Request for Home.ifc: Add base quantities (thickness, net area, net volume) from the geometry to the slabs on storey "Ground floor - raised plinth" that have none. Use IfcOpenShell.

First a look at what the model holds.

```python
import ifcopenshell
import ifcopenshell.util.element
import ifcopenshell.util.unit

model = ifcopenshell.open("Home.ifc")
print(model.schema)
for unit_type in ("LENGTHUNIT", "AREAUNIT", "VOLUMEUNIT"):
    print(unit_type, ifcopenshell.util.unit.calculate_unit_scale(model, unit_type))
storey = next(s for s in model.by_type("IfcBuildingStorey") if s.Name == "Ground floor - raised plinth")
slabs = [e for e in ifcopenshell.util.element.get_decomposition(storey) if e.is_a("IfcSlab")]
for e in sorted(slabs, key=lambda e: e.id()):
    print(e.id(), e.is_a(), e.Name, list(ifcopenshell.util.element.get_psets(e, qtos_only=True)), sep=" | ")
```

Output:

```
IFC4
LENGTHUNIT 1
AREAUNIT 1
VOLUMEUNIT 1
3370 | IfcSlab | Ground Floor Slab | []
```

```python
import ifcopenshell
import ifcopenshell.api.pset
import ifcopenshell.geom
import ifcopenshell.util.element
import ifcopenshell.util.shape
import ifcopenshell.util.unit

model = ifcopenshell.open("Home.ifc")
unit_scale = ifcopenshell.util.unit.calculate_unit_scale(model)
area_scale = ifcopenshell.util.unit.calculate_unit_scale(model, "AREAUNIT")
volume_scale = ifcopenshell.util.unit.calculate_unit_scale(model, "VOLUMEUNIT")
settings = ifcopenshell.geom.settings()

storey = next(s for s in model.by_type("IfcBuildingStorey") if s.Name == "Ground floor - raised plinth")
slabs = [e for e in ifcopenshell.util.element.get_decomposition(storey) if e.is_a("IfcSlab")]

for e in sorted(slabs, key=lambda e: e.id()):
    if ifcopenshell.util.element.get_psets(e, qtos_only=True, should_inherit=False):
        continue
    # Geometry comes back in metres, in the element's own axes.
    shape = ifcopenshell.geom.create_shape(settings, e)
    values = {
        "Width": ifcopenshell.util.shape.get_z(shape.geometry) / unit_scale,
        "NetArea": ifcopenshell.util.shape.get_footprint_area(shape.geometry) / area_scale,
        "NetVolume": ifcopenshell.util.shape.get_volume(shape.geometry) / volume_scale,
    }
    qto = ifcopenshell.api.pset.add_qto(model, product=e, name="Qto_SlabBaseQuantities")
    ifcopenshell.api.pset.edit_qto(model, qto=qto, properties=values)
    print(e.id(), {k: round(v, 3) for k, v in values.items()})

model.write("Home_v2.ifc")
```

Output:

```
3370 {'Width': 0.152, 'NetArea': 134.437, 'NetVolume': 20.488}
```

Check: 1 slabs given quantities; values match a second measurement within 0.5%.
